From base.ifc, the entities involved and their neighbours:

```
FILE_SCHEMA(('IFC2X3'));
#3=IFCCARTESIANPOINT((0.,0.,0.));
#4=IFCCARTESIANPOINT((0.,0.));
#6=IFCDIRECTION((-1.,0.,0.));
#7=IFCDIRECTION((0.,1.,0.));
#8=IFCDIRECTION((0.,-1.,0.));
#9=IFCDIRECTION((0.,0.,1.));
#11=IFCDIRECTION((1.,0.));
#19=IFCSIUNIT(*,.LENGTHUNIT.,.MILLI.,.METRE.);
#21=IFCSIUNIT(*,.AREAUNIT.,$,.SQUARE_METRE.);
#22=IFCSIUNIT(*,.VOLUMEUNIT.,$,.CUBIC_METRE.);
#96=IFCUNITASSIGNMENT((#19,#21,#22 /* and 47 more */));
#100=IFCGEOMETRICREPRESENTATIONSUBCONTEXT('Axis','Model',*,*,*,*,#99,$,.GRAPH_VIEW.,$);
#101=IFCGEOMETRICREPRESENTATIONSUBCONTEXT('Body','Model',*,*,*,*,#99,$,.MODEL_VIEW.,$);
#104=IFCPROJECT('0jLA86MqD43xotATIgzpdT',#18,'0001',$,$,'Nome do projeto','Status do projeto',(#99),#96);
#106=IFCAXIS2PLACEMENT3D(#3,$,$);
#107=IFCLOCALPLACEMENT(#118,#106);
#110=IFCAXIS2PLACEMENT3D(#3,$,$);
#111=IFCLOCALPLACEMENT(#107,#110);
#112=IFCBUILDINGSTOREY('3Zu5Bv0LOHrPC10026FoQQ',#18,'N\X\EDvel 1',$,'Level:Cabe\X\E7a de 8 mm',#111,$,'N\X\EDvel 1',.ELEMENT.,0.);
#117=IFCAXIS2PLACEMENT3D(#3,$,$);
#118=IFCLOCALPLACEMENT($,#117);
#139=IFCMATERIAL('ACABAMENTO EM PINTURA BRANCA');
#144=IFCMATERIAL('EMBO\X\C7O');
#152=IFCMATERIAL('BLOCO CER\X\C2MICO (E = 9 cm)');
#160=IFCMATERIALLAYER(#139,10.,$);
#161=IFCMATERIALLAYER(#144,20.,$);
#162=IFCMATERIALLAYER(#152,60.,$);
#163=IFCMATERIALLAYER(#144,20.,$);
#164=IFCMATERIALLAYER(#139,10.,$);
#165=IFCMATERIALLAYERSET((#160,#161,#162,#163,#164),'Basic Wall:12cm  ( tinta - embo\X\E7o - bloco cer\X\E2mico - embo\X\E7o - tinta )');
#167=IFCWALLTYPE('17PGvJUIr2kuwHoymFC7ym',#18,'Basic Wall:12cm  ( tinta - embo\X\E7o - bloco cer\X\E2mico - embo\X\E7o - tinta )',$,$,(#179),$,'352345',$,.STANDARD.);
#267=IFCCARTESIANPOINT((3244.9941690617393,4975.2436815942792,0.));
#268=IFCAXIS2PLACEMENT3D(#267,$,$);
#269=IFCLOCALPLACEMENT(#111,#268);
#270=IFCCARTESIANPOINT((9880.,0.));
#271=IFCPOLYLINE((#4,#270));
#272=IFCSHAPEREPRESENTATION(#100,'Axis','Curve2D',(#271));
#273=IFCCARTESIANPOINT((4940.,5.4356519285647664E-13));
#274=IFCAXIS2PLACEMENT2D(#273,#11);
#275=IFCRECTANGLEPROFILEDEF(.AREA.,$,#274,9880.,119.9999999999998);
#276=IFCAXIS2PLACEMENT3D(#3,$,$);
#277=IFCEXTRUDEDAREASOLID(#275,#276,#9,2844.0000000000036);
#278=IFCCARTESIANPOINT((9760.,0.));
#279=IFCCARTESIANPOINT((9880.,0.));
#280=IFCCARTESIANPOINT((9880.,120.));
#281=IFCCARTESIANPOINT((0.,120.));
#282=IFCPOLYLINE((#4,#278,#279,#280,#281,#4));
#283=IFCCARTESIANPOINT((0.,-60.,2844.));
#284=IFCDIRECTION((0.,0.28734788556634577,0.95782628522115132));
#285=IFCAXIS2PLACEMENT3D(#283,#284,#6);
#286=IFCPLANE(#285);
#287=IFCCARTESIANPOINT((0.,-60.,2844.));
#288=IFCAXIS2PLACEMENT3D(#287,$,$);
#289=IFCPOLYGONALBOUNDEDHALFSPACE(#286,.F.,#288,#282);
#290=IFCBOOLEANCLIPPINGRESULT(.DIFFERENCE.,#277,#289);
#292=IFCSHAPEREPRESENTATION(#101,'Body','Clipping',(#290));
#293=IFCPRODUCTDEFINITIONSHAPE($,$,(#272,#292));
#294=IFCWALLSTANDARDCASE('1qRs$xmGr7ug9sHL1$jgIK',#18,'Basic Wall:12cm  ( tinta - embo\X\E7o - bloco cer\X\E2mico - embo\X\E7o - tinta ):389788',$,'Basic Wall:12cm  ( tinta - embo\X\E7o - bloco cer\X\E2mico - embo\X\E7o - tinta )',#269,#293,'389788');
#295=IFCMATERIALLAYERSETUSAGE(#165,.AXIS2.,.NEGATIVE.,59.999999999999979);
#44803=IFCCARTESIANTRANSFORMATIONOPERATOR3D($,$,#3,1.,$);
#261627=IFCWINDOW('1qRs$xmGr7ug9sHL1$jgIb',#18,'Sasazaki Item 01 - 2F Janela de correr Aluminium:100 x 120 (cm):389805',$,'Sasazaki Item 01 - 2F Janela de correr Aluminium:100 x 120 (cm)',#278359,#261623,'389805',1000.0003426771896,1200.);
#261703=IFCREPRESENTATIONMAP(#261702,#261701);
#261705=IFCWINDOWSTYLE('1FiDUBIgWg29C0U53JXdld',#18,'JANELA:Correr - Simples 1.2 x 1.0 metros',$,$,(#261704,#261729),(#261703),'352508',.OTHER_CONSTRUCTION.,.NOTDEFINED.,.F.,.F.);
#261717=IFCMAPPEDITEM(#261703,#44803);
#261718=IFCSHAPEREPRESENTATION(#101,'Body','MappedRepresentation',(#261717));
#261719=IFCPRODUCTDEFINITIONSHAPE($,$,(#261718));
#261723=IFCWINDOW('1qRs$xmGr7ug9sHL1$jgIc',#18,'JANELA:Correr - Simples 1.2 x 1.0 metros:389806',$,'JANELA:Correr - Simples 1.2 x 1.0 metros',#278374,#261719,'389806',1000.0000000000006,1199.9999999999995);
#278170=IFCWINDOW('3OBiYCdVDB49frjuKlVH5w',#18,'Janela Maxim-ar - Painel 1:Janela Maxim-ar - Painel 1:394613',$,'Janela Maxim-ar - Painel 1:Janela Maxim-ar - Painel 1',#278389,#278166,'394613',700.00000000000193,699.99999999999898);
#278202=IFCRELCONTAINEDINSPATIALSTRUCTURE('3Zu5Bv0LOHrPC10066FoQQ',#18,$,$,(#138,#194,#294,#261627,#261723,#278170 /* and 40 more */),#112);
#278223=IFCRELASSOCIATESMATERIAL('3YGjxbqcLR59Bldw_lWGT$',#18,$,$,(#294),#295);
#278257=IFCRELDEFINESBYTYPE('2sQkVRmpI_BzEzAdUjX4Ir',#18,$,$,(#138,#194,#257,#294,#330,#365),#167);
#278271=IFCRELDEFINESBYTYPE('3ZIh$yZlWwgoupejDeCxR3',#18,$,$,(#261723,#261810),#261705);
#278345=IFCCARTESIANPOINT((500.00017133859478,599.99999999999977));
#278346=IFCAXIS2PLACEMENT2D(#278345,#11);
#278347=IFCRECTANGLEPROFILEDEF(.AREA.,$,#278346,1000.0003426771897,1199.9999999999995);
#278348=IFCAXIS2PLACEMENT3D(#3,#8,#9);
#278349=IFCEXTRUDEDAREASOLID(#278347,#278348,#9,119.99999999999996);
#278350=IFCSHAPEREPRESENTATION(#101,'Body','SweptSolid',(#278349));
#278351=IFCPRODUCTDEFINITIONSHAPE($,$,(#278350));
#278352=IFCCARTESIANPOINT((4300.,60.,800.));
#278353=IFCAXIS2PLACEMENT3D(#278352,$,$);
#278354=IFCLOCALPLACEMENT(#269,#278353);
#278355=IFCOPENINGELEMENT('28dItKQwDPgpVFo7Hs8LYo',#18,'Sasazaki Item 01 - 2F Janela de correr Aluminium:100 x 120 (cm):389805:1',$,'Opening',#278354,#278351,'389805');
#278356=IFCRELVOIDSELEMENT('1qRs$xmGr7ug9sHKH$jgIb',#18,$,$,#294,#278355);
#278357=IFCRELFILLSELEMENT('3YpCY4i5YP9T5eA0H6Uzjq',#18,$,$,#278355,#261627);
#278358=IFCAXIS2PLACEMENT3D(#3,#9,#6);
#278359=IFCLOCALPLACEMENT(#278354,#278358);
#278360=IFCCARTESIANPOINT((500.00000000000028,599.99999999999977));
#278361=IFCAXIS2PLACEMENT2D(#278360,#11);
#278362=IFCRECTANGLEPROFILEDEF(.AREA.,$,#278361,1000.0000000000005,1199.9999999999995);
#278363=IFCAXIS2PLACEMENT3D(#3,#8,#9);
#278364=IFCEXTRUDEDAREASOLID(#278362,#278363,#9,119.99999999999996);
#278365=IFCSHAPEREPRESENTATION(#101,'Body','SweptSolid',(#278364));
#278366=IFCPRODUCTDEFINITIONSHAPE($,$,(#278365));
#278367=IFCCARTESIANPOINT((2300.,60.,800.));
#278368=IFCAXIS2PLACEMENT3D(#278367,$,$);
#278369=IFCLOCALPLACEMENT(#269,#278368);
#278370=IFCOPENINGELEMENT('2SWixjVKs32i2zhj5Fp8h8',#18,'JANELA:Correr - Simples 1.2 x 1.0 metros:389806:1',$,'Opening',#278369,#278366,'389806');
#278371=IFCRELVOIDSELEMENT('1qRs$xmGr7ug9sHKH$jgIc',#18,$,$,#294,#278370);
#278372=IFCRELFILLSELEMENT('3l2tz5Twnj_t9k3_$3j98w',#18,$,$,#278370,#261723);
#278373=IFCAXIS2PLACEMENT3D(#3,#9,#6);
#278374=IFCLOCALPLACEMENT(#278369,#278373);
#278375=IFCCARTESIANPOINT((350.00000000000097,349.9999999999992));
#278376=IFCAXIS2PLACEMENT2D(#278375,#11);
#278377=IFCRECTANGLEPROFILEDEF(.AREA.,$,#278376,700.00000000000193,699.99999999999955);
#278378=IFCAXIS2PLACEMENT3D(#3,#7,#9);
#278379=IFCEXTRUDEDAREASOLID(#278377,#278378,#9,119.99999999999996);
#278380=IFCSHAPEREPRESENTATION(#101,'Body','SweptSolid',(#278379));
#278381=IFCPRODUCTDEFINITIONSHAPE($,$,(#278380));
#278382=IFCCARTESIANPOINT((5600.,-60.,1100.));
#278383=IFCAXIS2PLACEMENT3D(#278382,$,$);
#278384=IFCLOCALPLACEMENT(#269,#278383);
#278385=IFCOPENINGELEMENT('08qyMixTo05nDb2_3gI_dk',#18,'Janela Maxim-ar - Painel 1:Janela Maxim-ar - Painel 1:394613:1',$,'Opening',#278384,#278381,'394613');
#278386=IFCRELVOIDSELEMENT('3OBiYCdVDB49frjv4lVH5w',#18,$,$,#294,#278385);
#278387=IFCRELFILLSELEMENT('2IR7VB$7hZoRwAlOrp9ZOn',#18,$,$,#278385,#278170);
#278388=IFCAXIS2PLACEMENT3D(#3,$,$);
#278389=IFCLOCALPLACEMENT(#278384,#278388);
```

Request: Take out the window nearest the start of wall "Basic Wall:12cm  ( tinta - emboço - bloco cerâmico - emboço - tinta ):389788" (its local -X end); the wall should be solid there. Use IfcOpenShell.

```python
import ifcopenshell
import ifcopenshell.api.feature
import ifcopenshell.api.root
import ifcopenshell.geom
import ifcopenshell.util.shape

model = ifcopenshell.open("base.ifc")
settings = ifcopenshell.geom.settings()


def volume(element):
    """Net volume in cubic metres, openings subtracted."""
    shape = ifcopenshell.geom.create_shape(settings, element)
    return ifcopenshell.util.shape.get_volume(shape.geometry)


window = model.by_id(261723)
opening = window.FillsVoids[0].RelatingOpeningElement
wall = opening.VoidsElements[0].RelatingBuildingElement
before = volume(wall)

ifcopenshell.api.root.remove_product(model, product=window)
ifcopenshell.api.feature.remove_feature(model, feature=opening)

after = volume(wall)

print(f"wall volume {before:.3f} -> {after:.3f} m3")

model.write("base_rev.ifc")
```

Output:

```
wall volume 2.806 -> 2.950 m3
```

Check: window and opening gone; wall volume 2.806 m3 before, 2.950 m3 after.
